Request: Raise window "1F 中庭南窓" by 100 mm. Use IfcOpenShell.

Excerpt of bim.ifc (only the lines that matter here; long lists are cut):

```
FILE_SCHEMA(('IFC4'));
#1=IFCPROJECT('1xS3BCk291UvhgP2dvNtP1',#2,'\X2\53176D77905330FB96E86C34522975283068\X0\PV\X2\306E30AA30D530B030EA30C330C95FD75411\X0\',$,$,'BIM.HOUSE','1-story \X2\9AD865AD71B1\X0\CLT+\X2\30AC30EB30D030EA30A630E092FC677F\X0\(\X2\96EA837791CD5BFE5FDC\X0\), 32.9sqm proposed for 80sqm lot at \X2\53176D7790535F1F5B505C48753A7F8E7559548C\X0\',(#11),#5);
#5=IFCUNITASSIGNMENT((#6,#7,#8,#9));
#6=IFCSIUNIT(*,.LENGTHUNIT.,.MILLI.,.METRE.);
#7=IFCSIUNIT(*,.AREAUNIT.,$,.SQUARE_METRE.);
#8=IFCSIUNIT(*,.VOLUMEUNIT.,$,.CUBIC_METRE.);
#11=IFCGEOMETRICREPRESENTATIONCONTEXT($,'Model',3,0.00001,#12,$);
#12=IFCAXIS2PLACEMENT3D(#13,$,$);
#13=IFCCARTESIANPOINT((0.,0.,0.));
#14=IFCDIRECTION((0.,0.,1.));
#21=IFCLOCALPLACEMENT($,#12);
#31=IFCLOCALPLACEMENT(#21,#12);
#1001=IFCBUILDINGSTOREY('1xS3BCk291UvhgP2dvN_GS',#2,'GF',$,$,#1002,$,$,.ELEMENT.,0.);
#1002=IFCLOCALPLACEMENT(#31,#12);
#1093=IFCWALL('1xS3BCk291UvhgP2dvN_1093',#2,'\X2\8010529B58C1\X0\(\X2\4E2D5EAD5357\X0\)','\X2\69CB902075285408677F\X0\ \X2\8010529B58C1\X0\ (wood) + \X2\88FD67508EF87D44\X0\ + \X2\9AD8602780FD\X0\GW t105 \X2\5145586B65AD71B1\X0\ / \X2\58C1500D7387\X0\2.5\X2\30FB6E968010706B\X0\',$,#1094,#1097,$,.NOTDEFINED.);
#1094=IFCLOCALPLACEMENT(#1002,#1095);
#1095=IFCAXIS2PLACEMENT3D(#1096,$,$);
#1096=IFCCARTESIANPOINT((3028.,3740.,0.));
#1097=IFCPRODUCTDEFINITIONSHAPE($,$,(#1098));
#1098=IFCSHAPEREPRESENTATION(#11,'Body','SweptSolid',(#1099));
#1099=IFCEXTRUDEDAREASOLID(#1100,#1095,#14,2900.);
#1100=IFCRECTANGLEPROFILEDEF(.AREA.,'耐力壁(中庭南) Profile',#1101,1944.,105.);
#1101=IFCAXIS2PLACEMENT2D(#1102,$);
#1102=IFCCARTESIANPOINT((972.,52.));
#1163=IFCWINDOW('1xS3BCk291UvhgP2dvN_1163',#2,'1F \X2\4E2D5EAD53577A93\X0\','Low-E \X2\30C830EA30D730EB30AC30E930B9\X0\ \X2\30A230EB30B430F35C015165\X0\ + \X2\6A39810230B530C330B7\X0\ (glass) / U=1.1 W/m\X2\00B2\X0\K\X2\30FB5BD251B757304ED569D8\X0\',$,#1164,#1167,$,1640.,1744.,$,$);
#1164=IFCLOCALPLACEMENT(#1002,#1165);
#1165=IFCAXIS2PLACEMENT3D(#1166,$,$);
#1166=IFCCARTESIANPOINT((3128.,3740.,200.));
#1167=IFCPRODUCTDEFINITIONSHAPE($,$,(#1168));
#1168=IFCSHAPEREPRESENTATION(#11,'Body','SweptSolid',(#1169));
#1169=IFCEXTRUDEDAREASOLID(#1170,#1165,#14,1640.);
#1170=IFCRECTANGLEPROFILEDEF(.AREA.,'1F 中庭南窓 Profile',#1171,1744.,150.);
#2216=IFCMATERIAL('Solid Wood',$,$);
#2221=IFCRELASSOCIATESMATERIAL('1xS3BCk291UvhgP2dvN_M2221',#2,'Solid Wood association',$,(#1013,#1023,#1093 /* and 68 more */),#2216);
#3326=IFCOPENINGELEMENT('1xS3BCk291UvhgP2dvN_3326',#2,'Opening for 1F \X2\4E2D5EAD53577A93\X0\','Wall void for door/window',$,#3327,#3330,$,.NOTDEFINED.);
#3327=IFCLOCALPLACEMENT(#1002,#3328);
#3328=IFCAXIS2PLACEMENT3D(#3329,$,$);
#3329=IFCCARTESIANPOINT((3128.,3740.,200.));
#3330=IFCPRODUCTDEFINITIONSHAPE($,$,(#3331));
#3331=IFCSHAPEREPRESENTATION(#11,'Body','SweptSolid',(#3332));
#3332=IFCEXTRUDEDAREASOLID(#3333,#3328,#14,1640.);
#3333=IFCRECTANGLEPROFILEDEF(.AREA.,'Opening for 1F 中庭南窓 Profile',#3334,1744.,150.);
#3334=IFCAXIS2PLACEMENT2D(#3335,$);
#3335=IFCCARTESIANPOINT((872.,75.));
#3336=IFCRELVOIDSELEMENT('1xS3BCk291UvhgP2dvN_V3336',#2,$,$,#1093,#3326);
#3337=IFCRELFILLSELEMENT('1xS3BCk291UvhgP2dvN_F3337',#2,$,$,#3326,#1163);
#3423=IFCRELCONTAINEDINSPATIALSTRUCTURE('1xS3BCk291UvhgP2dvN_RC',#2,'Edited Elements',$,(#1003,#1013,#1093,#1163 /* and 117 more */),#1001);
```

```python
import numpy as np
import ifcopenshell
import ifcopenshell.api.geometry
import ifcopenshell.util.placement
import ifcopenshell.util.unit

model = ifcopenshell.open("bim.ifc")
unit_scale = ifcopenshell.util.unit.calculate_unit_scale(model)

window = model.by_guid("1xS3BCk291UvhgP2dvN_1163")
opening = window.FillsVoids[0].RelatingOpeningElement
dz = 0.1 / unit_scale

shift = np.array([0.0, 0.0, dz])
# The window is not placed relative to its opening, so move both.
for product in (opening, window):
    matrix = ifcopenshell.util.placement.get_local_placement(product.ObjectPlacement)
    matrix[:3, 3] += shift
    ifcopenshell.api.geometry.edit_object_placement(model, product=product, matrix=matrix, is_si=False)

print(f"moved by {dz * unit_scale:+.3f} m")

model.write("bim-out.ifc")
```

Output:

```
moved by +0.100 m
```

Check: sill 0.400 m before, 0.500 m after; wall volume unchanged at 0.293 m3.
